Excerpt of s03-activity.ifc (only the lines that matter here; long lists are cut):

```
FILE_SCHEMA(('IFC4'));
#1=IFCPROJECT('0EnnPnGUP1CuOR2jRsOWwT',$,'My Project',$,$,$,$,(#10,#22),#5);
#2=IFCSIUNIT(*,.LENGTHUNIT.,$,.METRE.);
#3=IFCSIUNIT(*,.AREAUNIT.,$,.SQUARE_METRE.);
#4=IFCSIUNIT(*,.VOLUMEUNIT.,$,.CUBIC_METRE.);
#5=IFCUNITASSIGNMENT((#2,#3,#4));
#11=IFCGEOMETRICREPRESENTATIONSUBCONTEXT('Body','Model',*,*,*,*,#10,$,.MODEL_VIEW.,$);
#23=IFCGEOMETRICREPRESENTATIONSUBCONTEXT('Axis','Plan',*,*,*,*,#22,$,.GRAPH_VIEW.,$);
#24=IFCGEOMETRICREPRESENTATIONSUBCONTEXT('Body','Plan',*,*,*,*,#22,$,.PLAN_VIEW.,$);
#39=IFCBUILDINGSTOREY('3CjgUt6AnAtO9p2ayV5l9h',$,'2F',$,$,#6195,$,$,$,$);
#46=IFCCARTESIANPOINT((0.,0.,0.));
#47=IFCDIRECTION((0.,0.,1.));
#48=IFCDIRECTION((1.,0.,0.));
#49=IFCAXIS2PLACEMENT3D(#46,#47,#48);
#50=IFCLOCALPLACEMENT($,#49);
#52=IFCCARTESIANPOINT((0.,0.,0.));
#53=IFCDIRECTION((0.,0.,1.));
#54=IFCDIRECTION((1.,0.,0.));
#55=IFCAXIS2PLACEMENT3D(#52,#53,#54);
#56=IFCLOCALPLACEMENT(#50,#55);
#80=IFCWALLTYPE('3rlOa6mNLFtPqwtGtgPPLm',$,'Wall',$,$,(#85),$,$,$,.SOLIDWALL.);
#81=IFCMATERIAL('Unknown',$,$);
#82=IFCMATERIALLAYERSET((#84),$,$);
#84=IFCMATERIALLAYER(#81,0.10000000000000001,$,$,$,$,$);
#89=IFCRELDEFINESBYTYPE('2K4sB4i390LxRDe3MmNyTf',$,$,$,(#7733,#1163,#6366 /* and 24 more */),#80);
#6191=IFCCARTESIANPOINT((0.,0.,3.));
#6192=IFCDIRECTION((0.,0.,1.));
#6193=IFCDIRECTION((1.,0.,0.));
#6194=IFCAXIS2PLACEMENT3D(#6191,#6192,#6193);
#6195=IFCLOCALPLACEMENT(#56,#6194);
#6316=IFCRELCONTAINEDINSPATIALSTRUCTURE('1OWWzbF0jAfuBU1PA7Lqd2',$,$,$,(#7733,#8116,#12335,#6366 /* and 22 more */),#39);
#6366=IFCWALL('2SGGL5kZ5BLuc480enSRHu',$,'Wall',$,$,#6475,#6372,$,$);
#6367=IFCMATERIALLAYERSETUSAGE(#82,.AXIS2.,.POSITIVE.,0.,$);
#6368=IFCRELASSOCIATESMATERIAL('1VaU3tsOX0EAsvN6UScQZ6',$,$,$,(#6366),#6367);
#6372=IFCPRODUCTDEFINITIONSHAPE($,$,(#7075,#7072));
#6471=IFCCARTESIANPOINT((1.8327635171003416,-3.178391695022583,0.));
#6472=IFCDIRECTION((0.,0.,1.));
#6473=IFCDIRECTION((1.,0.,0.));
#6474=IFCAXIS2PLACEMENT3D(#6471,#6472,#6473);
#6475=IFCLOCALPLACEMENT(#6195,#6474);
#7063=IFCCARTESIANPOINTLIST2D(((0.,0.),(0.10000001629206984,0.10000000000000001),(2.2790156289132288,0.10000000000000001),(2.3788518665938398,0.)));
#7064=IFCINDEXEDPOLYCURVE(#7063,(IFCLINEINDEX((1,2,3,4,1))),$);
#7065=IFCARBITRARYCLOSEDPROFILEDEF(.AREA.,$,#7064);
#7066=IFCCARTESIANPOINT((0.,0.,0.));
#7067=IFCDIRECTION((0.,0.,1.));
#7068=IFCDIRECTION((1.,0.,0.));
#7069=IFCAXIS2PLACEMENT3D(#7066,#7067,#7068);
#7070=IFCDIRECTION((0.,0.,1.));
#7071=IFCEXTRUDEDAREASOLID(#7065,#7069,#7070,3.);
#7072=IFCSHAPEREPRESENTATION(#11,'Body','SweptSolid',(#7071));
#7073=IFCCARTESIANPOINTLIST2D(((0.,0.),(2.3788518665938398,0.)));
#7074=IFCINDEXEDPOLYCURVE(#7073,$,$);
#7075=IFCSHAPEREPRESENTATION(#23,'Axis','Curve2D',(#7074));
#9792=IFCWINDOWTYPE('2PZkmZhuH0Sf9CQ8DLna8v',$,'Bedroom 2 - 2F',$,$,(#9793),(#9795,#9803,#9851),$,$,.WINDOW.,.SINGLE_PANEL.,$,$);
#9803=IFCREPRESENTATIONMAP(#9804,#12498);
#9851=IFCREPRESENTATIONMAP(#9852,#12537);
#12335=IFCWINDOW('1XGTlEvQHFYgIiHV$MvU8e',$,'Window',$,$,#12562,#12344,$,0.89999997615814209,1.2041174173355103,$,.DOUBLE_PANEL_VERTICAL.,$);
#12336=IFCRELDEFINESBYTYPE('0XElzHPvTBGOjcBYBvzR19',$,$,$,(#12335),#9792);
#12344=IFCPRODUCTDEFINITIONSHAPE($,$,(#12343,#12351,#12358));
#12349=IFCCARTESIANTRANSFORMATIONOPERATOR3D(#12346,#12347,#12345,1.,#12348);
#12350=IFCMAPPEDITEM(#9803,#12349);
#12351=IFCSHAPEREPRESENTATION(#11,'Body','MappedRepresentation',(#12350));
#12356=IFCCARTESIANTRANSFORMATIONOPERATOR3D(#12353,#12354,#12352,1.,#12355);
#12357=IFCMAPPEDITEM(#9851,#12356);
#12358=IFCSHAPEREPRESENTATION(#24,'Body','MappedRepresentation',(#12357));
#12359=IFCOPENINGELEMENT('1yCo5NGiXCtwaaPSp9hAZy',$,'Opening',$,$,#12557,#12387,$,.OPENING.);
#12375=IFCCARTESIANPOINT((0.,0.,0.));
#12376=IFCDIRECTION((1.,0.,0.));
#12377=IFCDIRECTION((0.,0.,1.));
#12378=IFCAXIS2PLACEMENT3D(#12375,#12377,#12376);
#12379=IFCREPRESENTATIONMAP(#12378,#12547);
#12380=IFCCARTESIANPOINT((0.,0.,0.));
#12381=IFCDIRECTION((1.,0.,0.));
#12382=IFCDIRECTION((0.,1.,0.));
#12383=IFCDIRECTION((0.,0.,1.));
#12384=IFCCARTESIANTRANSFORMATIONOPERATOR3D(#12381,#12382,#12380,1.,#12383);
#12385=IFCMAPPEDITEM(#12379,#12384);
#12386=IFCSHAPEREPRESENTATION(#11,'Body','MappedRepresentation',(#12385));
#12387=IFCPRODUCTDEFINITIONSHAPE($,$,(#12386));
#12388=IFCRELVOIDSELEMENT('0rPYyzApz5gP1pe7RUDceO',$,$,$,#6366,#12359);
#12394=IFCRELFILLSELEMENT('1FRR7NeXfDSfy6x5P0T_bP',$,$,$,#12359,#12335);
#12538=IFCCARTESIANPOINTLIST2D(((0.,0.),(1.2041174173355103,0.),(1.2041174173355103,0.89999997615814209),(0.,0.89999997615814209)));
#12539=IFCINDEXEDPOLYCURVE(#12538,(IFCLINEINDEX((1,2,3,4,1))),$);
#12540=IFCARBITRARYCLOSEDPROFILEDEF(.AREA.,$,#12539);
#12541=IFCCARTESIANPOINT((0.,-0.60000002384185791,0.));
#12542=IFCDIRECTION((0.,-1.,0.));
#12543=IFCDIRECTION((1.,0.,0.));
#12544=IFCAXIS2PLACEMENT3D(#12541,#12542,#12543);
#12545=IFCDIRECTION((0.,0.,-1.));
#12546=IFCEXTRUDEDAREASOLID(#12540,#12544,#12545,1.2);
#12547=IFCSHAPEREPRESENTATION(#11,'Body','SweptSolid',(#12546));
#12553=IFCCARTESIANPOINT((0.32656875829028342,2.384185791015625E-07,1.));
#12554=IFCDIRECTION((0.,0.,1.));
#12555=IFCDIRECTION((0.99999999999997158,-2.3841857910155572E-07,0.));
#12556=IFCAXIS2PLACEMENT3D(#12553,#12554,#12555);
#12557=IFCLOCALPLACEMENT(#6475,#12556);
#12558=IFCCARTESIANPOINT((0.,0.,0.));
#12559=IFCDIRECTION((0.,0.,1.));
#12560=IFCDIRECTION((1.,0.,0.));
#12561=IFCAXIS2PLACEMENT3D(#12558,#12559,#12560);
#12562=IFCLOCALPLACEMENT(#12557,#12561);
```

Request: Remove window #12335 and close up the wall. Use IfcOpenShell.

```python
import ifcopenshell
import ifcopenshell.api.feature
import ifcopenshell.api.root
import ifcopenshell.geom
import ifcopenshell.util.shape

model = ifcopenshell.open("s03-activity.ifc")
settings = ifcopenshell.geom.settings()


def volume(element):
    """Net volume in cubic metres, openings subtracted."""
    shape = ifcopenshell.geom.create_shape(settings, element)
    return ifcopenshell.util.shape.get_volume(shape.geometry)


window = model.by_id(12335)
opening = window.FillsVoids[0].RelatingOpeningElement
wall = opening.VoidsElements[0].RelatingBuildingElement
before = volume(wall)

ifcopenshell.api.root.remove_product(model, product=window)
ifcopenshell.api.feature.remove_feature(model, feature=opening)

after = volume(wall)

print(f"wall volume {before:.3f} -> {after:.3f} m3")

model.write("s03-activity_rev.ifc")
```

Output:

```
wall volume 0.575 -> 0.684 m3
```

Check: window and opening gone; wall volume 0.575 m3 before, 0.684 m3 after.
